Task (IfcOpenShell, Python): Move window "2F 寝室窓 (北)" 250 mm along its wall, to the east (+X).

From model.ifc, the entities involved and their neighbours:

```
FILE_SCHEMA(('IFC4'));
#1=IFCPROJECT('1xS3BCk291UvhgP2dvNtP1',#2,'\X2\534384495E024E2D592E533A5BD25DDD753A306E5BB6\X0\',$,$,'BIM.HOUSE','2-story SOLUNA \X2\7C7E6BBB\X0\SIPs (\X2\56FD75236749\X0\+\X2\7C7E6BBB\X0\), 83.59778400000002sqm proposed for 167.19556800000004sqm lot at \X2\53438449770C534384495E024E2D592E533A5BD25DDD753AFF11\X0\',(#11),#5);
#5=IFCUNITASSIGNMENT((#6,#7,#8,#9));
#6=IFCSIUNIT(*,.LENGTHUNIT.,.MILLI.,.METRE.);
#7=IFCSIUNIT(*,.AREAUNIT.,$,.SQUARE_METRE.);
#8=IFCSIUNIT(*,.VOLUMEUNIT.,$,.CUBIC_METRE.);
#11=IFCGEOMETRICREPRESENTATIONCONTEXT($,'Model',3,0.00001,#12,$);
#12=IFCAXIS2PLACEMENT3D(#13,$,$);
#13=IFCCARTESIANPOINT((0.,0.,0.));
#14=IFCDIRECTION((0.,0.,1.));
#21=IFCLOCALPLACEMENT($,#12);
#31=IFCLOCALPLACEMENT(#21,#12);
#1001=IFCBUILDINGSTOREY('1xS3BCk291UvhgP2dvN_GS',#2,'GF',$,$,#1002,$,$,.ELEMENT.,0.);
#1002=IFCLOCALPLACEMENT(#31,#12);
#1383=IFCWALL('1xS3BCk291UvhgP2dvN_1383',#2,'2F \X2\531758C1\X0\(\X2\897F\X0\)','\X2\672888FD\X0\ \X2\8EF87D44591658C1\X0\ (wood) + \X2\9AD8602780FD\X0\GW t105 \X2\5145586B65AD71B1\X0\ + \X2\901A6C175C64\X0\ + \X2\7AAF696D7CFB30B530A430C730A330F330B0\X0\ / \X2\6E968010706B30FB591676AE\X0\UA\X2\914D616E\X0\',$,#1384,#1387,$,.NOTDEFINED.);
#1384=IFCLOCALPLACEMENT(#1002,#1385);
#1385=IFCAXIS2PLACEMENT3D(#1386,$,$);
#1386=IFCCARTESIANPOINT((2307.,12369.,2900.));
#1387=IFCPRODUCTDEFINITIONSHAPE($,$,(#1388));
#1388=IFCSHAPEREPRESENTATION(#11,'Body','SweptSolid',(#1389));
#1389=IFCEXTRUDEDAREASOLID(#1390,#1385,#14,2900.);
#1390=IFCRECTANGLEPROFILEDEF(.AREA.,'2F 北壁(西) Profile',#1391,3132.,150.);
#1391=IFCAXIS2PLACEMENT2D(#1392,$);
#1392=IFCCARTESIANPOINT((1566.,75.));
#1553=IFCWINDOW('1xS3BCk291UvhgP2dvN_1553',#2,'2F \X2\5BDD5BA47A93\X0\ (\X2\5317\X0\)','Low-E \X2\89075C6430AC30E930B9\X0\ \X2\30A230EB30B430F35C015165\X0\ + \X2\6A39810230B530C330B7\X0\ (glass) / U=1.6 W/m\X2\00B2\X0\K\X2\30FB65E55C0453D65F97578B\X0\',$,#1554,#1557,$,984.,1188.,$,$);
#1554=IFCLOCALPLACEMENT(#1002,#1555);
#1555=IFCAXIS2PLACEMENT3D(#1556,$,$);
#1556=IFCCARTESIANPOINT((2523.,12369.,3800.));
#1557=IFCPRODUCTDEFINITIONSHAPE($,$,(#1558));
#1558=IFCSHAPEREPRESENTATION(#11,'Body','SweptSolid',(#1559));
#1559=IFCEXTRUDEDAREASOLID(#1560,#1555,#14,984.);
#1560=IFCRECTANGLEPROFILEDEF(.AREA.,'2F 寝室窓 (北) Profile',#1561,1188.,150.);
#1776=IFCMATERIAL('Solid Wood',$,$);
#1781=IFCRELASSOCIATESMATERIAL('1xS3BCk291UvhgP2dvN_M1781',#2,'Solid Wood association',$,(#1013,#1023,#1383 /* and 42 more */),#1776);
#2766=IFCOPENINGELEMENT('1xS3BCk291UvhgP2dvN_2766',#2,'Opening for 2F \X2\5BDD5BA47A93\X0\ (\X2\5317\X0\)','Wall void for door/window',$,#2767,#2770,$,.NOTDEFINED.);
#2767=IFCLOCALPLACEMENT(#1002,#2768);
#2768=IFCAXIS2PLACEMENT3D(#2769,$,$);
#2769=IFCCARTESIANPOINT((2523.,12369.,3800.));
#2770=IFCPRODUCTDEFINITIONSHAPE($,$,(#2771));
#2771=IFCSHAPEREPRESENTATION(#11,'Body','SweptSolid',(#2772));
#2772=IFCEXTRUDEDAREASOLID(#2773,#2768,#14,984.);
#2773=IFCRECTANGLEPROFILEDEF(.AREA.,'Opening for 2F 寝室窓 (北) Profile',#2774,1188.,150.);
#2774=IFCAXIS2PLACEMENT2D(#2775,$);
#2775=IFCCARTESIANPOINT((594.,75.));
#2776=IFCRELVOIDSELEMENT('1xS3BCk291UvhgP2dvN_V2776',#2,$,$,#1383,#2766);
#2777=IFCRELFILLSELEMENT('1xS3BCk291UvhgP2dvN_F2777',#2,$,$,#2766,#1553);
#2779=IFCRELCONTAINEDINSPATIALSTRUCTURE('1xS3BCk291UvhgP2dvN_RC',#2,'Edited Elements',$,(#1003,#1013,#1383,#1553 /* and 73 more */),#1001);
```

```python
import ifcopenshell
import ifcopenshell.api.geometry
import ifcopenshell.util.placement

model = ifcopenshell.open("model.ifc")

window = model.by_guid("1xS3BCk291UvhgP2dvN_1553")
opening = window.FillsVoids[0].RelatingOpeningElement
wall = opening.VoidsElements[0].RelatingBuildingElement

wall_matrix = ifcopenshell.util.placement.get_local_placement(wall.ObjectPlacement)
shift = wall_matrix[:3, 0] * 250.0
before = ifcopenshell.util.placement.get_local_placement(window.ObjectPlacement)[:3, 3].copy()

# The window is not placed relative to its opening, so move both.
for product in (opening, window):
    matrix = ifcopenshell.util.placement.get_local_placement(product.ObjectPlacement)
    matrix[:3, 3] += shift
    ifcopenshell.api.geometry.edit_object_placement(model, product=product, matrix=matrix, is_si=False)

after = ifcopenshell.util.placement.get_local_placement(window.ObjectPlacement)[:3, 3]
print("window moved by", (after - before).round(3) + 0.0)

model.write("model-out.ifc")
```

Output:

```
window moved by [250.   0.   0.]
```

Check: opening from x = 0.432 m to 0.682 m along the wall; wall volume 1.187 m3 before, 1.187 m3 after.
